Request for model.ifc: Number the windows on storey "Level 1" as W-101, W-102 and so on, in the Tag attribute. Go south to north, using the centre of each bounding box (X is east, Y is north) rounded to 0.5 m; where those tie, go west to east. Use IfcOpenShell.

First a look at what the model holds.

```python
import ifcopenshell
import ifcopenshell.util.element
import ifcopenshell.util.placement

model = ifcopenshell.open("model.ifc")
print(model.schema)
storey = next(s for s in model.by_type("IfcBuildingStorey") if s.Name == "Level 1")
windows = [e for e in ifcopenshell.util.element.get_decomposition(storey) if e.is_a("IfcWindow")]
for e in sorted(windows, key=lambda e: e.id()):
    origin = ifcopenshell.util.placement.get_local_placement(e.ObjectPlacement)[:3, 3]
    print(e.id(), e.Tag, e.Name, origin.round(2) + 0.0, sep=" | ")
```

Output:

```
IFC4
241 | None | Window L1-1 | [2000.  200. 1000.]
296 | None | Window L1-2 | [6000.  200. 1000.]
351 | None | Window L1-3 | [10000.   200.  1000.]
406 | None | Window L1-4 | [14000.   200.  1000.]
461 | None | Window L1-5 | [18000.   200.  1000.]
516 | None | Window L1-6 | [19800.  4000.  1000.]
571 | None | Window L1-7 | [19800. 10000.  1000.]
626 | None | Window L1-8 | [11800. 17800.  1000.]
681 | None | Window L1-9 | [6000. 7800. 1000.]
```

```python
import ifcopenshell
import ifcopenshell.geom
import ifcopenshell.util.element
import ifcopenshell.util.shape

model = ifcopenshell.open("model.ifc")
settings = ifcopenshell.geom.settings()
settings.set("use-world-coords", True)


def centre(element):
    shape = ifcopenshell.geom.create_shape(settings, element)
    return ifcopenshell.util.shape.get_bbox_centroid(shape.geometry)


storey = next(s for s in model.by_type("IfcBuildingStorey") if s.Name == "Level 1")
windows = [e for e in ifcopenshell.util.element.get_decomposition(storey) if e.is_a("IfcWindow")]

# Insertion points can sit at a corner or the storey origin, so sort by the geometry (in metres).
centres = {e: centre(e) for e in windows}
windows.sort(key=lambda e: (round(centres[e][1] / 0.5), centres[e][0]))

for i, e in enumerate(windows, start=1):
    number = f"W-1{i:02d}"
    e.Tag = number
    print(e.id(), number)

model.write("model_rev.ifc")
```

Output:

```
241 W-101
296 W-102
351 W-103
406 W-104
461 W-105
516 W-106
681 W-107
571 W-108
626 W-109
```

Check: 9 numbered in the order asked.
